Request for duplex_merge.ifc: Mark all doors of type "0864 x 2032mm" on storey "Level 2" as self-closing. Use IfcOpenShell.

First a look at what the model holds.

```python
import ifcopenshell
import ifcopenshell.util.element

model = ifcopenshell.open("duplex_merge.ifc")
print(model.schema)
storey = next(s for s in model.by_type("IfcBuildingStorey") if s.Name == "Level 2")
doors = [e for e in ifcopenshell.util.element.get_decomposition(storey) if e.is_a("IfcDoor")]
seen = {}
for e in doors:
    element_type = ifcopenshell.util.element.get_type(e)
    key = (element_type.Name if element_type != e and element_type else None, ifcopenshell.util.element.get_pset(e, "Pset_DoorCommon", "SelfClosing"))
    seen[key] = seen.get(key, 0) + 1
for (name, value), count in sorted(seen.items(), key=str):
    print(count, "x", name, "|", value)
```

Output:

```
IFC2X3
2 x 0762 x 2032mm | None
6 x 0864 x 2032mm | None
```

```python
import ifcopenshell
import ifcopenshell.api.pset
import ifcopenshell.util.element

model = ifcopenshell.open("duplex_merge.ifc")

storey = next(s for s in model.by_type("IfcBuildingStorey") if s.Name == "Level 2")
doors = [e for e in ifcopenshell.util.element.get_decomposition(storey) if e.is_a("IfcDoor")]

count = 0
for e in doors:
    element_type = ifcopenshell.util.element.get_type(e)
    if element_type in (None, e) or element_type.Name != "0864 x 2032mm":
        continue
    # add_pset returns the element's existing set when there is one.
    pset = ifcopenshell.api.pset.add_pset(model, product=e, name="Pset_DoorCommon")
    ifcopenshell.api.pset.edit_pset(model, pset=pset, properties={"SelfClosing": True})
    count += 1

print(count, "doors updated")

model.write("duplex_merge_rev.ifc")
```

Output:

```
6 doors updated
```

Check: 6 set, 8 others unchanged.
